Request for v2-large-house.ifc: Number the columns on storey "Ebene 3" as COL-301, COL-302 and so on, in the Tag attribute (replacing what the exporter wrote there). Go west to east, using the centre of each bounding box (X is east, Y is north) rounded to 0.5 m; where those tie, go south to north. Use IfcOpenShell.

First a look at what the model holds.

```python
import ifcopenshell
import ifcopenshell.util.element
import ifcopenshell.util.placement

model = ifcopenshell.open("v2-large-house.ifc")
print(model.schema)
storey = next(s for s in model.by_type("IfcBuildingStorey") if s.Name == "Ebene 3")
columns = [e for e in ifcopenshell.util.element.get_decomposition(storey) if e.is_a("IfcColumn")]
for e in sorted(columns, key=lambda e: e.id()):
    origin = ifcopenshell.util.placement.get_local_placement(e.ObjectPlacement)[:3, 3]
    print(e.id(), e.Tag, e.Name, origin.round(2) + 0.0, sep=" | ")
```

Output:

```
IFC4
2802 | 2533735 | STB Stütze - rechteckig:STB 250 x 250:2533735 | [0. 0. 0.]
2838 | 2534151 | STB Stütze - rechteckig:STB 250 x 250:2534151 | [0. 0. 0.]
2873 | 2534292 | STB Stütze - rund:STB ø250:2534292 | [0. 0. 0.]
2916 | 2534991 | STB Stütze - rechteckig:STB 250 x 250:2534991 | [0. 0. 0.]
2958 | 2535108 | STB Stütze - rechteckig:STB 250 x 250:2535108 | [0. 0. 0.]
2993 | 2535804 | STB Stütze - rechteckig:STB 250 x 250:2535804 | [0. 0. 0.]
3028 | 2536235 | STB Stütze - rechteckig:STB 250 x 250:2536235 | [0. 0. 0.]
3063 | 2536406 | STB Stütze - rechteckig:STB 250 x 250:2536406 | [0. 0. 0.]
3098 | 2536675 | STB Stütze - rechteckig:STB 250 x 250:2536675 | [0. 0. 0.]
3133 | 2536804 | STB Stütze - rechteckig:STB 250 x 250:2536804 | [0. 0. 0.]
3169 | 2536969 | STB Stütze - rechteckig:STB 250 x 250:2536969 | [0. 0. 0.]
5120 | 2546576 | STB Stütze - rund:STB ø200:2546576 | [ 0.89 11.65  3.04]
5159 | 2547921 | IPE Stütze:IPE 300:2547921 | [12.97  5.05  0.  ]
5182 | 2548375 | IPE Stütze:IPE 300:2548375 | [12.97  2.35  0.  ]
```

```python
import ifcopenshell
import ifcopenshell.geom
import ifcopenshell.util.element
import ifcopenshell.util.shape

model = ifcopenshell.open("v2-large-house.ifc")
settings = ifcopenshell.geom.settings()
settings.set("use-world-coords", True)


def centre(element):
    shape = ifcopenshell.geom.create_shape(settings, element)
    return ifcopenshell.util.shape.get_bbox_centroid(shape.geometry)


storey = next(s for s in model.by_type("IfcBuildingStorey") if s.Name == "Ebene 3")
columns = [e for e in ifcopenshell.util.element.get_decomposition(storey) if e.is_a("IfcColumn")]

# Insertion points can sit at a corner or the storey origin, so sort by the geometry (in metres).
centres = {e: centre(e) for e in columns}
columns.sort(key=lambda e: (round(centres[e][0] / 0.5), centres[e][1]))

for i, e in enumerate(columns, start=1):
    number = f"COL-3{i:02d}"
    e.Tag = number
    print(e.id(), number)

model.write("v2-large-house_edited.ifc")
```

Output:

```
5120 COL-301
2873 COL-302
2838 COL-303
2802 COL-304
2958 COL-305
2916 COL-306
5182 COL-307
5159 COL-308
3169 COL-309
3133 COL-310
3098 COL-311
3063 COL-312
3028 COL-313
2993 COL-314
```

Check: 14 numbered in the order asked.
